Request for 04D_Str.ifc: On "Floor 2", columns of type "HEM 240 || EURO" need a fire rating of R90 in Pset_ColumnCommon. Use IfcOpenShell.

First a look at what the model holds.

```python
import ifcopenshell
import ifcopenshell.util.element

model = ifcopenshell.open("04D_Str.ifc")
print(model.schema)
storey = next(s for s in model.by_type("IfcBuildingStorey") if s.Name == "Floor 2")
columns = [e for e in ifcopenshell.util.element.get_decomposition(storey) if e.is_a("IfcColumn")]
seen = {}
for e in columns:
    element_type = ifcopenshell.util.element.get_type(e)
    key = (element_type.Name if element_type != e and element_type else None, ifcopenshell.util.element.get_pset(e, "Pset_ColumnCommon", "FireRating"))
    seen[key] = seen.get(key, 0) + 1
for (name, value), count in sorted(seen.items(), key=str):
    print(count, "x", name, "|", value)
```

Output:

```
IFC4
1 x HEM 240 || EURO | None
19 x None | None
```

```python
import ifcopenshell
import ifcopenshell.api.pset
import ifcopenshell.util.element

model = ifcopenshell.open("04D_Str.ifc")

storey = next(s for s in model.by_type("IfcBuildingStorey") if s.Name == "Floor 2")
columns = [e for e in ifcopenshell.util.element.get_decomposition(storey) if e.is_a("IfcColumn")]

count = 0
for e in columns:
    element_type = ifcopenshell.util.element.get_type(e)
    if element_type in (None, e) or element_type.Name != "HEM 240 || EURO":
        continue
    # add_pset returns the element's existing set when there is one.
    pset = ifcopenshell.api.pset.add_pset(model, product=e, name="Pset_ColumnCommon")
    ifcopenshell.api.pset.edit_pset(model, pset=pset, properties={"FireRating": "R90"})
    count += 1

print(count, "columns updated")

model.write("04D_Str_rev.ifc")
```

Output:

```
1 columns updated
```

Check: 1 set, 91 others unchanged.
